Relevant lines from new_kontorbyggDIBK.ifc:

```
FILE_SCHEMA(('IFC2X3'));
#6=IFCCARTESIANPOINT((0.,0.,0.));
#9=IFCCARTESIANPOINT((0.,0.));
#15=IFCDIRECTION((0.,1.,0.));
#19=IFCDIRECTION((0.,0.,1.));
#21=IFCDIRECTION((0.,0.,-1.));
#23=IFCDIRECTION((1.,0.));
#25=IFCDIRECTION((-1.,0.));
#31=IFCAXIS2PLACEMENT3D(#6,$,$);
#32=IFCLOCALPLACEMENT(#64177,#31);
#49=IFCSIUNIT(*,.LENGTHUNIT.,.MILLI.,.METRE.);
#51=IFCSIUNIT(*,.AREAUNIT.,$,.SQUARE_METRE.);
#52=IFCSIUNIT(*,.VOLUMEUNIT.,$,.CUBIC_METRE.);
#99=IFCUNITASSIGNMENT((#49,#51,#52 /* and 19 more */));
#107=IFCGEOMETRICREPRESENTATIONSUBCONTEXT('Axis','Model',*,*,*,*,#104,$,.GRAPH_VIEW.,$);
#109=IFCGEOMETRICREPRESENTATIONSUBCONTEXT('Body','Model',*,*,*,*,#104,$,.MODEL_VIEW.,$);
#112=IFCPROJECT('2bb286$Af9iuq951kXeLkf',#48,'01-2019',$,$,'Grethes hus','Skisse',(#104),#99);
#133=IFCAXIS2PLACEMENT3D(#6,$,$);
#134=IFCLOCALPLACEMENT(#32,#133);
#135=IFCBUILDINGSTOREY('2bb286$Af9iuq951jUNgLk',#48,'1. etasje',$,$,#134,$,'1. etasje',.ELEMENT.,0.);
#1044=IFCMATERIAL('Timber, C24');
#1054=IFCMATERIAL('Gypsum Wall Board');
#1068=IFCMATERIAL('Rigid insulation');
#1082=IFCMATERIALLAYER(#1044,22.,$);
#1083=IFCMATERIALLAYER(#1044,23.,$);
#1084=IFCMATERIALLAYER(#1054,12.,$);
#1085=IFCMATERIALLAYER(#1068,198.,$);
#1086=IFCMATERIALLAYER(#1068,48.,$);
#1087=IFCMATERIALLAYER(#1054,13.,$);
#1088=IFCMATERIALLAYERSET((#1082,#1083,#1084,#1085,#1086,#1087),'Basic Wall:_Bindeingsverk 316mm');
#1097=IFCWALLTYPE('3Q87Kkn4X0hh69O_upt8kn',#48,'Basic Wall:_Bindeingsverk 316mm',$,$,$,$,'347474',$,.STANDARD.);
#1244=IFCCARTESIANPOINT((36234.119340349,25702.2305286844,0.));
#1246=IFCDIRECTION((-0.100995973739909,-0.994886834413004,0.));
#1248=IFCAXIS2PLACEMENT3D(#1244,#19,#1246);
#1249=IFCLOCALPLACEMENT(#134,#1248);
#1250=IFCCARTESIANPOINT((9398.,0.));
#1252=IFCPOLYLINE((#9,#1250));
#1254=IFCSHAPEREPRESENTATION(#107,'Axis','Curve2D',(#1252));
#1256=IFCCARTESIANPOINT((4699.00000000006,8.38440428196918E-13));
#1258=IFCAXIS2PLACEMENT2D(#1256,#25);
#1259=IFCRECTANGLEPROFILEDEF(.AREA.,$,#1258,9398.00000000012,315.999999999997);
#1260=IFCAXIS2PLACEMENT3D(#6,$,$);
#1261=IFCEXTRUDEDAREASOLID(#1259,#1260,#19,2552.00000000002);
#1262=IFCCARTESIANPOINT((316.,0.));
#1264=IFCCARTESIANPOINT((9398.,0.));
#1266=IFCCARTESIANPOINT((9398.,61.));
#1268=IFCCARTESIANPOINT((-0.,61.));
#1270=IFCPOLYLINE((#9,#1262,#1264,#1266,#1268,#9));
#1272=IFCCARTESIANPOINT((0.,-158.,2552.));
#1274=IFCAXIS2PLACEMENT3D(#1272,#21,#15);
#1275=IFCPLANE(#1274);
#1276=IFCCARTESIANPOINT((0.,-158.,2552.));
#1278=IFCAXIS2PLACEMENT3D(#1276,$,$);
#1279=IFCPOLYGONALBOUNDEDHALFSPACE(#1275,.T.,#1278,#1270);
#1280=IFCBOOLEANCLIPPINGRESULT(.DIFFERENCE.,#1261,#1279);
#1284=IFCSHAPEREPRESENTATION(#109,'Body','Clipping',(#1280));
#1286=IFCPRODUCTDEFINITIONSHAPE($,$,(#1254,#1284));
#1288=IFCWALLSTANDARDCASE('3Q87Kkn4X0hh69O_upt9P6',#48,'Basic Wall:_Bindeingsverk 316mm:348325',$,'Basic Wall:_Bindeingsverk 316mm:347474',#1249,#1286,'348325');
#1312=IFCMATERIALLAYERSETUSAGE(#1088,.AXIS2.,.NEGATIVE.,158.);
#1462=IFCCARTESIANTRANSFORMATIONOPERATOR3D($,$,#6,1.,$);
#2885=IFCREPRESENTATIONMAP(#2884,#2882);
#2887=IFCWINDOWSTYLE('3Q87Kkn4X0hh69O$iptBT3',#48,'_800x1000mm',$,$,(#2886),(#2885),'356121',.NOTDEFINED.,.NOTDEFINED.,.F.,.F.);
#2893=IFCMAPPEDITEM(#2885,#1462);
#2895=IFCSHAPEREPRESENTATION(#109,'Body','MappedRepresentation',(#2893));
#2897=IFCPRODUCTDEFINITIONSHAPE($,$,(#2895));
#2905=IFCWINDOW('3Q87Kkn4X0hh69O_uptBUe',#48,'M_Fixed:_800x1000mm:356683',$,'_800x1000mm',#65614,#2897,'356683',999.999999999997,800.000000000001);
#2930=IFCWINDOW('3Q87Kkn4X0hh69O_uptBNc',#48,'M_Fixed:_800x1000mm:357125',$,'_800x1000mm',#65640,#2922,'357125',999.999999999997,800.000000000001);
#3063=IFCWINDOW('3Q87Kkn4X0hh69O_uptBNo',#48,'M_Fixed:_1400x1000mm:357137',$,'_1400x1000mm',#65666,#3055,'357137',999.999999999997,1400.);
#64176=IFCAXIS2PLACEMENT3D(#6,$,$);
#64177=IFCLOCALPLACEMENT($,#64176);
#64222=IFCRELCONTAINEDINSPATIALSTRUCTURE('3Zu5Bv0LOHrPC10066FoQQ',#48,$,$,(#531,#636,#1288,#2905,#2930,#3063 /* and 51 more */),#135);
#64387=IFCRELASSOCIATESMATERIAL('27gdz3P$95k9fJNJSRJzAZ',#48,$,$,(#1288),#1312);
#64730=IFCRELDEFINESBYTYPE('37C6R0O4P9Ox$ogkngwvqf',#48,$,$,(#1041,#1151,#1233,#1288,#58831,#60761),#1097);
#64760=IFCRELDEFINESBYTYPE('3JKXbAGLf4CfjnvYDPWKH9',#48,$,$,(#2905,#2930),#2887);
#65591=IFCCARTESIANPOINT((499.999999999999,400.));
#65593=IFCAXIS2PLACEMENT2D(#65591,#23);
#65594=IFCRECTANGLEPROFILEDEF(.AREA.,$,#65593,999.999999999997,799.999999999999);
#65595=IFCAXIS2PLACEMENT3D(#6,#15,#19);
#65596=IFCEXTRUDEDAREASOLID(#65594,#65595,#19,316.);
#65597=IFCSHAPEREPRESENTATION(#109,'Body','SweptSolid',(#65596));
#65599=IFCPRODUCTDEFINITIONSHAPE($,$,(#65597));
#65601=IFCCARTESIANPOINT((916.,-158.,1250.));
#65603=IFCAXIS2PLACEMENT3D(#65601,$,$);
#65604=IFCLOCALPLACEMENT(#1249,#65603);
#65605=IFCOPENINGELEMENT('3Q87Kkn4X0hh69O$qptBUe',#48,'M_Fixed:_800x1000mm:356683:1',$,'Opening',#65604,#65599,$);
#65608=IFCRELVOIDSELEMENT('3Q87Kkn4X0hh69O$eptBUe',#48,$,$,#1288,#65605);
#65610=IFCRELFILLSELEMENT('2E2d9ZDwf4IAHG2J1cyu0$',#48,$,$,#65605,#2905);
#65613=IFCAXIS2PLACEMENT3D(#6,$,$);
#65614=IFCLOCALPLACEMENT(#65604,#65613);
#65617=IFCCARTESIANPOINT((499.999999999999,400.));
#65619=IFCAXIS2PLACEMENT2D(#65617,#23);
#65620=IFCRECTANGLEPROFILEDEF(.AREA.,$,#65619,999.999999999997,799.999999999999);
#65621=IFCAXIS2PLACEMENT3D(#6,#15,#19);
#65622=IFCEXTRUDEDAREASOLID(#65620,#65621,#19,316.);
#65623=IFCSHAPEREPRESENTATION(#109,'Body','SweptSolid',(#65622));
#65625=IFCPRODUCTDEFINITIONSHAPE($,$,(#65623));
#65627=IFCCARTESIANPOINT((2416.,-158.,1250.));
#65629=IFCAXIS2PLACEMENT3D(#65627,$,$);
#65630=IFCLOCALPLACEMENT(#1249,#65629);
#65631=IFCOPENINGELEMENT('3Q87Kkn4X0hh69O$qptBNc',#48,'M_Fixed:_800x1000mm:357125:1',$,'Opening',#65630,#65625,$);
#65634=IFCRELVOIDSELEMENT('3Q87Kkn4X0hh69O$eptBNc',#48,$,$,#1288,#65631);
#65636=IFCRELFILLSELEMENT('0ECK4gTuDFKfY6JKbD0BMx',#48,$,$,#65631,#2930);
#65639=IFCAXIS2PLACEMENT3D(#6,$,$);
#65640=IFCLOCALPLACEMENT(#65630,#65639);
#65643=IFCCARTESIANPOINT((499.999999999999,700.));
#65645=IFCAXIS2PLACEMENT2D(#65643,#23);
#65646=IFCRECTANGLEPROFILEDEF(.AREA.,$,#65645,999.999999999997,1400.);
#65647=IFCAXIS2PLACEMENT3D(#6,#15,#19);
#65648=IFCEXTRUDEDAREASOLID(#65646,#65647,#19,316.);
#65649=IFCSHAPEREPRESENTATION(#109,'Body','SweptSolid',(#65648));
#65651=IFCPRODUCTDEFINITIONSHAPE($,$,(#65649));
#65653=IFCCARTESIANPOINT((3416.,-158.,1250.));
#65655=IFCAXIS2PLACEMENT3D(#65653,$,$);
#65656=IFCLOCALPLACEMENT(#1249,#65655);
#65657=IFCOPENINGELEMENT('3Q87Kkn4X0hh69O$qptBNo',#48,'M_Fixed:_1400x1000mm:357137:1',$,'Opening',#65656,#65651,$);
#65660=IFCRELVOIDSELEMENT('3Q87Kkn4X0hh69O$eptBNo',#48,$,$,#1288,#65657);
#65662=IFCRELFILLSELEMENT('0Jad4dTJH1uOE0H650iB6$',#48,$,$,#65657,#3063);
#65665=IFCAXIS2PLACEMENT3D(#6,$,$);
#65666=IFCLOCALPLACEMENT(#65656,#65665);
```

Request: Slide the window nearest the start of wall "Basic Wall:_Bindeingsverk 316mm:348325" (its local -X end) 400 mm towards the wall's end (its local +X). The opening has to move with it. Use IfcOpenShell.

```python
import ifcopenshell
import ifcopenshell.api.geometry
import ifcopenshell.util.placement

model = ifcopenshell.open("new_kontorbyggDIBK.ifc")

window = model.by_id(2905)
opening = window.FillsVoids[0].RelatingOpeningElement
wall = opening.VoidsElements[0].RelatingBuildingElement

wall_matrix = ifcopenshell.util.placement.get_local_placement(wall.ObjectPlacement)
shift = wall_matrix[:3, 0] * 400.0
before = ifcopenshell.util.placement.get_local_placement(window.ObjectPlacement)[:3, 3].copy()

# The window is placed relative to its opening, so it follows when the opening moves.
matrix = ifcopenshell.util.placement.get_local_placement(opening.ObjectPlacement)
matrix[:3, 3] += shift
ifcopenshell.api.geometry.edit_object_placement(
    model, product=opening, matrix=matrix, is_si=False, should_transform_children=True
)

after = ifcopenshell.util.placement.get_local_placement(window.ObjectPlacement)[:3, 3]
print("window moved by", (after - before).round(3) + 0.0)

model.write("new_kontorbyggDIBK_edited.ifc")
```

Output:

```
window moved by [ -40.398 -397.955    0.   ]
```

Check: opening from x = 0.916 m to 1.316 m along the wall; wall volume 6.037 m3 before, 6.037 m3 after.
